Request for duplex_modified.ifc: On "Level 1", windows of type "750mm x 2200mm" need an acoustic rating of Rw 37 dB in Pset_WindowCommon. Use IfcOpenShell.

First a look at what the model holds.

```python
import ifcopenshell
import ifcopenshell.util.element

model = ifcopenshell.open("duplex_modified.ifc")
print(model.schema)
storey = next(s for s in model.by_type("IfcBuildingStorey") if s.Name == "Level 1")
windows = [e for e in ifcopenshell.util.element.get_decomposition(storey) if e.is_a("IfcWindow")]
seen = {}
for e in windows:
    element_type = ifcopenshell.util.element.get_type(e)
    key = (element_type.Name if element_type != e and element_type else None, ifcopenshell.util.element.get_pset(e, "Pset_WindowCommon", "AcousticRating"))
    seen[key] = seen.get(key, 0) + 1
for (name, value), count in sorted(seen.items(), key=str):
    print(count, "x", name, "|", value)
```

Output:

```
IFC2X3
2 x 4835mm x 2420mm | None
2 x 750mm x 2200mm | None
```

```python
import ifcopenshell
import ifcopenshell.api.pset
import ifcopenshell.util.element

model = ifcopenshell.open("duplex_modified.ifc")

storey = next(s for s in model.by_type("IfcBuildingStorey") if s.Name == "Level 1")
windows = [e for e in ifcopenshell.util.element.get_decomposition(storey) if e.is_a("IfcWindow")]

count = 0
for e in windows:
    element_type = ifcopenshell.util.element.get_type(e)
    if element_type in (None, e) or element_type.Name != "750mm x 2200mm":
        continue
    # add_pset returns the element's existing set when there is one.
    pset = ifcopenshell.api.pset.add_pset(model, product=e, name="Pset_WindowCommon")
    ifcopenshell.api.pset.edit_pset(model, pset=pset, properties={"AcousticRating": "Rw 37 dB"})
    count += 1

print(count, "windows updated")

model.write("duplex_modified_edited.ifc")
```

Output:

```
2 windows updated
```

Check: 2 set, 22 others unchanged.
